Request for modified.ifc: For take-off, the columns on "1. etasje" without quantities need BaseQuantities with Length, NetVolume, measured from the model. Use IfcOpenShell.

First a look at what the model holds.

```python
import ifcopenshell
import ifcopenshell.util.element
import ifcopenshell.util.unit

model = ifcopenshell.open("modified.ifc")
print(model.schema)
for unit_type in ("LENGTHUNIT", "AREAUNIT", "VOLUMEUNIT"):
    print(unit_type, ifcopenshell.util.unit.calculate_unit_scale(model, unit_type))
storey = next(s for s in model.by_type("IfcBuildingStorey") if s.Name == "1. etasje")
columns = [e for e in ifcopenshell.util.element.get_decomposition(storey) if e.is_a("IfcColumn")]
for e in sorted(columns, key=lambda e: e.id()):
    print(e.id(), e.is_a(), e.Name, list(ifcopenshell.util.element.get_psets(e, qtos_only=True)), sep=" | ")
```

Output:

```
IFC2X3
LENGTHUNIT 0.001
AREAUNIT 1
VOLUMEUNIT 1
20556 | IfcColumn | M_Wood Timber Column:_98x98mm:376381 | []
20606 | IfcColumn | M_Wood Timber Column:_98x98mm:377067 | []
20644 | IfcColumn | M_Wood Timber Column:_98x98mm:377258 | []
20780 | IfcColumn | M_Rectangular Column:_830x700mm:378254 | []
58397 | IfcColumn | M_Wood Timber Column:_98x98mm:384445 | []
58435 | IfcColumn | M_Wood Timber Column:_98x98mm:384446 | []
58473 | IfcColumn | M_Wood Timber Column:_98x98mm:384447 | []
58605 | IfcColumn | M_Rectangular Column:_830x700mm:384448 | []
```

```python
import ifcopenshell
import ifcopenshell.api.pset
import ifcopenshell.geom
import ifcopenshell.util.element
import ifcopenshell.util.shape
import ifcopenshell.util.unit

model = ifcopenshell.open("modified.ifc")
unit_scale = ifcopenshell.util.unit.calculate_unit_scale(model)
volume_scale = ifcopenshell.util.unit.calculate_unit_scale(model, "VOLUMEUNIT")
settings = ifcopenshell.geom.settings()

storey = next(s for s in model.by_type("IfcBuildingStorey") if s.Name == "1. etasje")
columns = [e for e in ifcopenshell.util.element.get_decomposition(storey) if e.is_a("IfcColumn")]

for e in sorted(columns, key=lambda e: e.id()):
    if ifcopenshell.util.element.get_psets(e, qtos_only=True, should_inherit=False):
        continue
    # Geometry comes back in metres, in the element's own axes.
    shape = ifcopenshell.geom.create_shape(settings, e)
    values = {
        "Length": ifcopenshell.util.shape.get_z(shape.geometry) / unit_scale,
        "NetVolume": ifcopenshell.util.shape.get_volume(shape.geometry) / volume_scale,
    }
    qto = ifcopenshell.api.pset.add_qto(model, product=e, name="BaseQuantities")
    ifcopenshell.api.pset.edit_qto(model, qto=qto, properties=values)
    print(e.id(), {k: round(v, 3) for k, v in values.items()})

model.write("modified_rev.ifc")
```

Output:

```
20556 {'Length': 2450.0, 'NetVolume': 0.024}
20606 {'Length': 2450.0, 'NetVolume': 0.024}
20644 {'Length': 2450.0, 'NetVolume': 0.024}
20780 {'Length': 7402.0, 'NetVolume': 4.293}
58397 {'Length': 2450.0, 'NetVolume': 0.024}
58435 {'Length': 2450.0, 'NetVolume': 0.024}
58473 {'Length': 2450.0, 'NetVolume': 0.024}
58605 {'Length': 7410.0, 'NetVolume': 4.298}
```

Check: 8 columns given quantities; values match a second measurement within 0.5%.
